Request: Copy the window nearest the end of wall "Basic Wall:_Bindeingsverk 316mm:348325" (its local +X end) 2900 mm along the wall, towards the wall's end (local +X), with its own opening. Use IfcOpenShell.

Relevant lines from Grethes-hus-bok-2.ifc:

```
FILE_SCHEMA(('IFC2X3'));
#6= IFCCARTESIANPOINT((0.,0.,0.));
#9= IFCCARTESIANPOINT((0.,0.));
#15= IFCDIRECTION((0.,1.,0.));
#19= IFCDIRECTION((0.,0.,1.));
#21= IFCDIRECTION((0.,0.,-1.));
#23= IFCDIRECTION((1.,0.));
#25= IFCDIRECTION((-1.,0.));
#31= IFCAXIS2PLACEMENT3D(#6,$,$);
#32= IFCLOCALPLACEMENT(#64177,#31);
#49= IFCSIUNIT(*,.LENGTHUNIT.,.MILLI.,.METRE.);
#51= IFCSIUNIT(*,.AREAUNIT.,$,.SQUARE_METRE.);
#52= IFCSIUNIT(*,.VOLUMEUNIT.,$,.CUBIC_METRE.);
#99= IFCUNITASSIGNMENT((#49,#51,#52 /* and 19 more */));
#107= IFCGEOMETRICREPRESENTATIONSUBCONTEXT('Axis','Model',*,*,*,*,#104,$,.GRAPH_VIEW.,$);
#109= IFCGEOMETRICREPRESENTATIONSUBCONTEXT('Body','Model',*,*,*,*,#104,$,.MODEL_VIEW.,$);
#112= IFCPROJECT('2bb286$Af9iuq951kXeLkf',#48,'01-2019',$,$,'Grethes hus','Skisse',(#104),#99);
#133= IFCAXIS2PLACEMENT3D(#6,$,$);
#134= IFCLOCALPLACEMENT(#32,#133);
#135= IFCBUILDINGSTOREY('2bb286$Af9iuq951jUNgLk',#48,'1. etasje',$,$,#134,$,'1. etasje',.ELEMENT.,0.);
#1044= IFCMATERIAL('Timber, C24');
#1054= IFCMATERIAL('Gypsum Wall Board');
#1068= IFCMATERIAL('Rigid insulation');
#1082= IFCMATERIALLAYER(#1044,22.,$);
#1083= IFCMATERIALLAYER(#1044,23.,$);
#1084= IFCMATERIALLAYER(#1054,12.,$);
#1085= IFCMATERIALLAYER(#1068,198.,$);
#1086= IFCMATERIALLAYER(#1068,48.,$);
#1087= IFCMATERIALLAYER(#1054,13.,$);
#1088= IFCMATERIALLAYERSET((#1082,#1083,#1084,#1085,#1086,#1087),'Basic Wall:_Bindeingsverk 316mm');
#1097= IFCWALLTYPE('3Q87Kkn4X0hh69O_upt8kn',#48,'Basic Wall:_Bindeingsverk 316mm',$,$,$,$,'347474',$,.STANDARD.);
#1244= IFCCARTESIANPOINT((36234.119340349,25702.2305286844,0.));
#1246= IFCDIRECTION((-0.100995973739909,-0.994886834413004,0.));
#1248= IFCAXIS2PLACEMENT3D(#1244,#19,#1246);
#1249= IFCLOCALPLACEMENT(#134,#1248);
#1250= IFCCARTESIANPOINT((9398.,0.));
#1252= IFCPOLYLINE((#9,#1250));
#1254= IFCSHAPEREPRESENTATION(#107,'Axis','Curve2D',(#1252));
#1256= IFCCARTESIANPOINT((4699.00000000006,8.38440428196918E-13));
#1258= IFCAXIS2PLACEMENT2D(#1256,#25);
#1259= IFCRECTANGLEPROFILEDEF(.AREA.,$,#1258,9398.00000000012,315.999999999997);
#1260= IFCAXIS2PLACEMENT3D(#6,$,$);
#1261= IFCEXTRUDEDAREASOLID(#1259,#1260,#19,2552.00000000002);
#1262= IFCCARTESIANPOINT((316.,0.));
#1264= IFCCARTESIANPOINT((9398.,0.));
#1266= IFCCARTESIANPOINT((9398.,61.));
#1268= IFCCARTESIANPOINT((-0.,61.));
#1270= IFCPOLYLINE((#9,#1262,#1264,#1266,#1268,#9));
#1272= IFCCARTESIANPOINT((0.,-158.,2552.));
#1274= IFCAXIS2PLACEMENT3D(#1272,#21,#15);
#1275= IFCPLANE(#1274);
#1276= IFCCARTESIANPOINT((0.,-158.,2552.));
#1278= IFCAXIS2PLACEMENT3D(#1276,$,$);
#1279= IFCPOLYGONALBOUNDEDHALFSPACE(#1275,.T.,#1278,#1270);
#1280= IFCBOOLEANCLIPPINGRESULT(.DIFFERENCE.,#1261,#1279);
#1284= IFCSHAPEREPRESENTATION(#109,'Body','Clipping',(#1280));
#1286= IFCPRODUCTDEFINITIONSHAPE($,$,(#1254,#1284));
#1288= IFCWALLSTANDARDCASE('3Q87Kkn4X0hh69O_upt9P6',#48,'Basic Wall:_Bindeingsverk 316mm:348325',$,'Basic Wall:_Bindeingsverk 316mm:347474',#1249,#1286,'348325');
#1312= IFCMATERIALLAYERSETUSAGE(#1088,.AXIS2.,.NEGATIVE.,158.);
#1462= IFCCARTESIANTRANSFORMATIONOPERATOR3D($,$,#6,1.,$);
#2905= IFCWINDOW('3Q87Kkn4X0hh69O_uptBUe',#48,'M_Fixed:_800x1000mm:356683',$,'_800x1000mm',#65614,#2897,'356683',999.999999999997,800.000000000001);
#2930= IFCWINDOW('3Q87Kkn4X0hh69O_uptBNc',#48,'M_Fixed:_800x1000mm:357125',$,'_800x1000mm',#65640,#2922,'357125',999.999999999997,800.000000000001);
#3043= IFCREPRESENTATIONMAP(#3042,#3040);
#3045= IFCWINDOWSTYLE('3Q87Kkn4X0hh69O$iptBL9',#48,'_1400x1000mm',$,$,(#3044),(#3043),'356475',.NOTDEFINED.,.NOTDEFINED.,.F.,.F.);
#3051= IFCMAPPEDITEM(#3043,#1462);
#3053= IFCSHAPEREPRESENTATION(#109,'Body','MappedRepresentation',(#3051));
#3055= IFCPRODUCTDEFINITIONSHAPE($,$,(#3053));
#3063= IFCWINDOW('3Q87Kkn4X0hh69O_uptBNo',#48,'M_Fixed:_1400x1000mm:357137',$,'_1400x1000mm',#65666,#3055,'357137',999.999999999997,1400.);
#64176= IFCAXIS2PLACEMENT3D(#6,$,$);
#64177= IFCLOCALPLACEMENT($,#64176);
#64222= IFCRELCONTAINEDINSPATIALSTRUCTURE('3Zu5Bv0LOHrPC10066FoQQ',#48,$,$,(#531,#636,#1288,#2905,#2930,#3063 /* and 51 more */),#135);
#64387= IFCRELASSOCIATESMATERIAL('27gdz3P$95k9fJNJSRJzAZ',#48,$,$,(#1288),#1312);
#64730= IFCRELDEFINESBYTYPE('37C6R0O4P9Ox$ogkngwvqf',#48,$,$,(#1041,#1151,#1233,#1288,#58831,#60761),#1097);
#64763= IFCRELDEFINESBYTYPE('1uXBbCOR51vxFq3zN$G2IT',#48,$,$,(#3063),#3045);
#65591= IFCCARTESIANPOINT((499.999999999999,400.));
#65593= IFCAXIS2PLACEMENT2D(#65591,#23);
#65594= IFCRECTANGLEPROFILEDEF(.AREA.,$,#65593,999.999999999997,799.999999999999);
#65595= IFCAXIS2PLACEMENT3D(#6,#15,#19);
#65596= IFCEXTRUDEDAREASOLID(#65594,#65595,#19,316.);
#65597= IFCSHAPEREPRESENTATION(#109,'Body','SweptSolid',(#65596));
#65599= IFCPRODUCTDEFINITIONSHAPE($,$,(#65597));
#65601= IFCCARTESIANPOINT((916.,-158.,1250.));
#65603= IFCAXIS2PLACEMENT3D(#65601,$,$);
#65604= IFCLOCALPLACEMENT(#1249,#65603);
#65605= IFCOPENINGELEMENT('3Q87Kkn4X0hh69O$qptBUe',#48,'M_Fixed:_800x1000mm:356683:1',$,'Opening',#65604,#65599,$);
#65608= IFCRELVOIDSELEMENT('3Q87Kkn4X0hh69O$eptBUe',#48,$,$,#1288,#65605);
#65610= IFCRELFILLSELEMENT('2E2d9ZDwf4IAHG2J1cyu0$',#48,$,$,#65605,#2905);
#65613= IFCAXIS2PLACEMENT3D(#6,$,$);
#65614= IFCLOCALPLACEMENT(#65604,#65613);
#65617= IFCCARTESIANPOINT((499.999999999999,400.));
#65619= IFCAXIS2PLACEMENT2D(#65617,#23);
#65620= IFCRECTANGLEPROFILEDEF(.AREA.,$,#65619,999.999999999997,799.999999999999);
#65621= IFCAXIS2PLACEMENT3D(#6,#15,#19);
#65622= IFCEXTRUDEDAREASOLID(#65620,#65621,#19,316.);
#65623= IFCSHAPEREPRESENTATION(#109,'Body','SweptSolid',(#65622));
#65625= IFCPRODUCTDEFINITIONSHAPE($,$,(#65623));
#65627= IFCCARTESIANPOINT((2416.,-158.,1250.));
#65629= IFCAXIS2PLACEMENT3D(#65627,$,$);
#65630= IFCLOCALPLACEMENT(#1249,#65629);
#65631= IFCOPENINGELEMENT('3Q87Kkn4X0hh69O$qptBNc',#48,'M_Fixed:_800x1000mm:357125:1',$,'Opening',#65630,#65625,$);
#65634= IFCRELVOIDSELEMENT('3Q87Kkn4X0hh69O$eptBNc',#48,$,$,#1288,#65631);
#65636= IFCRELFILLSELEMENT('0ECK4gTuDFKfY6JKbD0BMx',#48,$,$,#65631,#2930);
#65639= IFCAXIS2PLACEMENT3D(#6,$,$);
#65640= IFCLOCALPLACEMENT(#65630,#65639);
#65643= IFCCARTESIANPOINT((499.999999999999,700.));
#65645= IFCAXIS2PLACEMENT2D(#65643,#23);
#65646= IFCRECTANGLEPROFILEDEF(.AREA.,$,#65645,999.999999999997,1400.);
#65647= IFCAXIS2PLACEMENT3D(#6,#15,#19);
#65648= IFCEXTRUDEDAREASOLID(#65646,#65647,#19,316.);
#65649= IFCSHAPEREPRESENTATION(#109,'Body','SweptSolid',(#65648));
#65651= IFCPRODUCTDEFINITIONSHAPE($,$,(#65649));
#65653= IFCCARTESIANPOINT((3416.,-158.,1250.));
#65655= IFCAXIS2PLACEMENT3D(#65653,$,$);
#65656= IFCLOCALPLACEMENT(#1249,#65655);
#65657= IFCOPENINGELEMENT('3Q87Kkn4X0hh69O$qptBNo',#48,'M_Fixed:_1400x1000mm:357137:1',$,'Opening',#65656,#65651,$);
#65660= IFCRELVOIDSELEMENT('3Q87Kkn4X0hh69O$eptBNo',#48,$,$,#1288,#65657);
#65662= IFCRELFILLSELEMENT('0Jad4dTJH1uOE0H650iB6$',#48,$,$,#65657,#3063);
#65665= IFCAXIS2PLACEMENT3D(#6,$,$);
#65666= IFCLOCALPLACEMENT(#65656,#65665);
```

```python
import ifcopenshell
import ifcopenshell.api.feature
import ifcopenshell.api.geometry
import ifcopenshell.api.root
import ifcopenshell.geom
import ifcopenshell.util.element
import ifcopenshell.util.placement
import ifcopenshell.util.shape
import ifcopenshell.util.unit

model = ifcopenshell.open("Grethes-hus-bok-2.ifc")
unit_scale = ifcopenshell.util.unit.calculate_unit_scale(model)
settings = ifcopenshell.geom.settings()


def volume(element):
    """Net volume in cubic metres, openings subtracted."""
    shape = ifcopenshell.geom.create_shape(settings, element)
    return ifcopenshell.util.shape.get_volume(shape.geometry)


def reuse_history(source, copy):
    """copy_class also copies each property set's owner history, people and application; keep the originals."""
    for rel in copy.IsDefinedBy:
        if rel.is_a("IfcRelDefinesByProperties") and (history := rel.RelatingPropertyDefinition.OwnerHistory):
            rel.RelatingPropertyDefinition.OwnerHistory = source.OwnerHistory
            ifcopenshell.util.element.remove_deep2(model, history)


window = model.by_guid("3Q87Kkn4X0hh69O_uptBNo")
opening = window.FillsVoids[0].RelatingOpeningElement
wall = opening.VoidsElements[0].RelatingBuildingElement
before = volume(wall)
shift = ifcopenshell.util.placement.get_local_placement(wall.ObjectPlacement)[:3, 0] * 2.9 / unit_scale

# copy_class copies the void relationship, type, container and properties, but no geometry.
new_opening = ifcopenshell.api.root.copy_class(model, product=opening)
new_opening.Representation = ifcopenshell.util.element.copy_deep(
    model, opening.Representation, exclude=["IfcGeometricRepresentationContext", "IfcRepresentationMap"]
)
new_opening.Name = "M_Fixed:_1400x1000mm"
new_window = ifcopenshell.api.root.copy_class(model, product=window)
new_window.Representation = ifcopenshell.util.element.copy_deep(
    model, window.Representation, exclude=["IfcGeometricRepresentationContext", "IfcRepresentationMap"]
)
new_window.Name = "M_Fixed:_1400x1000mm"
new_window.Tag = None
reuse_history(window, new_window)
fills = ifcopenshell.api.feature.add_filling(model, opening=new_opening, element=new_window)
fills.OwnerHistory = new_window.OwnerHistory  # required in IFC2X3

for old, new in ((opening, new_opening), (window, new_window)):
    matrix = ifcopenshell.util.placement.get_local_placement(old.ObjectPlacement)
    matrix[:3, 3] += shift
    ifcopenshell.api.geometry.edit_object_placement(model, product=new, matrix=matrix, is_si=False)

after = volume(wall)

print(f"wall volume {before:.3f} -> {after:.3f} m3")

model.write("Grethes-hus-bok-2_updated.ifc")
```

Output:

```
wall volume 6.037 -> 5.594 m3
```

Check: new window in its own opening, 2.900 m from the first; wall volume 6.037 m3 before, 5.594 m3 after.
